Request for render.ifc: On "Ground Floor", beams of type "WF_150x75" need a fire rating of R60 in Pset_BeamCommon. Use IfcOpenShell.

First a look at what the model holds.

```python
import ifcopenshell
import ifcopenshell.util.element

model = ifcopenshell.open("render.ifc")
print(model.schema)
storey = next(s for s in model.by_type("IfcBuildingStorey") if s.Name == "Ground Floor")
beams = [e for e in ifcopenshell.util.element.get_decomposition(storey) if e.is_a("IfcBeam")]
seen = {}
for e in beams:
    element_type = ifcopenshell.util.element.get_type(e)
    key = (element_type.Name if element_type != e and element_type else None, ifcopenshell.util.element.get_pset(e, "Pset_BeamCommon", "FireRating"))
    seen[key] = seen.get(key, 0) + 1
for (name, value), count in sorted(seen.items(), key=str):
    print(count, "x", name, "|", value)
```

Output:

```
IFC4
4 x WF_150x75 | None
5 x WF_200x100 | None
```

```python
import ifcopenshell
import ifcopenshell.api.pset
import ifcopenshell.util.element

model = ifcopenshell.open("render.ifc")

storey = next(s for s in model.by_type("IfcBuildingStorey") if s.Name == "Ground Floor")
beams = [e for e in ifcopenshell.util.element.get_decomposition(storey) if e.is_a("IfcBeam")]

count = 0
for e in beams:
    element_type = ifcopenshell.util.element.get_type(e)
    if element_type in (None, e) or element_type.Name != "WF_150x75":
        continue
    # add_pset returns the element's existing set when there is one.
    pset = ifcopenshell.api.pset.add_pset(model, product=e, name="Pset_BeamCommon")
    ifcopenshell.api.pset.edit_pset(model, pset=pset, properties={"FireRating": "R60"})
    count += 1

print(count, "beams updated")

model.write("render_v2.ifc")
```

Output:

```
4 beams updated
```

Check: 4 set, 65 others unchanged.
